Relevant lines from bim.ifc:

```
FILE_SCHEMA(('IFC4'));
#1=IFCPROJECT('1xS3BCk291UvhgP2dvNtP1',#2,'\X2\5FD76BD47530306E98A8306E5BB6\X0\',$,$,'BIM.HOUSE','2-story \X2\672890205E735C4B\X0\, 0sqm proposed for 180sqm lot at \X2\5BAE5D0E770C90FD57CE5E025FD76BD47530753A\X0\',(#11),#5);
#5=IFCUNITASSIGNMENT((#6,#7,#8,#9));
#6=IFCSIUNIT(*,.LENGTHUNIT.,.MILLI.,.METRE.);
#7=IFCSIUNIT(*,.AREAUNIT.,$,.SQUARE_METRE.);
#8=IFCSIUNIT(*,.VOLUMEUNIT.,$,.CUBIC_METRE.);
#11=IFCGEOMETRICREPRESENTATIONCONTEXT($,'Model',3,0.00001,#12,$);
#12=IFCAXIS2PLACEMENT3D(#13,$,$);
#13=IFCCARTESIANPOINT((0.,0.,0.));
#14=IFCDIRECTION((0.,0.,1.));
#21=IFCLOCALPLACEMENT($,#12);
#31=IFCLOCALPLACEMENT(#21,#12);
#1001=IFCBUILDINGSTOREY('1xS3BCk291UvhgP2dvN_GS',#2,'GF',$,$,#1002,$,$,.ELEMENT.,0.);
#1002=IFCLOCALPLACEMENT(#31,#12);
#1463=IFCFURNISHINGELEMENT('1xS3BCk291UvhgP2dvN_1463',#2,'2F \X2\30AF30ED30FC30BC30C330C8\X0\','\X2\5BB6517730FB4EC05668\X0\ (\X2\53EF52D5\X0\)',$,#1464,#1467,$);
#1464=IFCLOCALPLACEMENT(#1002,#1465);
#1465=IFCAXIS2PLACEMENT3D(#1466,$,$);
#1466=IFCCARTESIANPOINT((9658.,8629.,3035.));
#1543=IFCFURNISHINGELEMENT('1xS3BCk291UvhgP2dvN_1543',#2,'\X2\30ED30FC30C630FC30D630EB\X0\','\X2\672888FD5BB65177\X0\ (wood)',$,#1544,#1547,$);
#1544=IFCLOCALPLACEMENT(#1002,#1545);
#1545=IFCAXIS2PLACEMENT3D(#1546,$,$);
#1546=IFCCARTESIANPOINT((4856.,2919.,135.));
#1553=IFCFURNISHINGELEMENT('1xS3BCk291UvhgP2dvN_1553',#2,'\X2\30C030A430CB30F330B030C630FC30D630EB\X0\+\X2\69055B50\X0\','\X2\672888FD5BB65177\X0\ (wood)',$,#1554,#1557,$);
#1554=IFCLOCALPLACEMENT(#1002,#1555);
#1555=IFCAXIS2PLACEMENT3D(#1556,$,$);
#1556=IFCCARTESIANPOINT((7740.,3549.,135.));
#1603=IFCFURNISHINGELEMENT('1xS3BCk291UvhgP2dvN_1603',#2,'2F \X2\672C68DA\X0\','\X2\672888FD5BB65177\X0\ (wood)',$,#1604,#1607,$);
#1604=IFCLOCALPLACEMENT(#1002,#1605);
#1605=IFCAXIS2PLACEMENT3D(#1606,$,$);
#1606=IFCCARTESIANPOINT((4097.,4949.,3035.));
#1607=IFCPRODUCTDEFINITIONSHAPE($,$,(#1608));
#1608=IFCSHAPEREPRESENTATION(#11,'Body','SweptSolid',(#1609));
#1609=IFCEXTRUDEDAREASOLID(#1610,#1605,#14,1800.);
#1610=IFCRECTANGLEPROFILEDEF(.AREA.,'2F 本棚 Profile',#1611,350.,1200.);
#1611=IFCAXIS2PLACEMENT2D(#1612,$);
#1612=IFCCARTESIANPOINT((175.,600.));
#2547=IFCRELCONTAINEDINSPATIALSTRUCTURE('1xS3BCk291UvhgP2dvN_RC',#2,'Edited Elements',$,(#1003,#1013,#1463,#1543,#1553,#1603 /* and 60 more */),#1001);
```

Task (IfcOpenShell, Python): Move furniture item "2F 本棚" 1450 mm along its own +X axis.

```python
import ifcopenshell
import ifcopenshell.api.geometry
import ifcopenshell.util.placement
import ifcopenshell.util.unit

model = ifcopenshell.open("bim.ifc")
unit_scale = ifcopenshell.util.unit.calculate_unit_scale(model)

item = model.by_guid("1xS3BCk291UvhgP2dvN_1603")
matrix = ifcopenshell.util.placement.get_local_placement(item.ObjectPlacement)
matrix[:3, 3] += matrix[:3, 0] * 1.45 / unit_scale
ifcopenshell.api.geometry.edit_object_placement(model, product=item, matrix=matrix, is_si=False)

print(ifcopenshell.util.placement.get_local_placement(item.ObjectPlacement).round(3) + 0.0)

model.write("bim_updated.ifc")
```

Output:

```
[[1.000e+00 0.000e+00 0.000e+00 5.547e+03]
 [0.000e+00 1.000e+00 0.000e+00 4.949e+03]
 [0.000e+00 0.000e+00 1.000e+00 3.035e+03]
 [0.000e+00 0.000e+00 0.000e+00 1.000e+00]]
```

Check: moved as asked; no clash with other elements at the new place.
